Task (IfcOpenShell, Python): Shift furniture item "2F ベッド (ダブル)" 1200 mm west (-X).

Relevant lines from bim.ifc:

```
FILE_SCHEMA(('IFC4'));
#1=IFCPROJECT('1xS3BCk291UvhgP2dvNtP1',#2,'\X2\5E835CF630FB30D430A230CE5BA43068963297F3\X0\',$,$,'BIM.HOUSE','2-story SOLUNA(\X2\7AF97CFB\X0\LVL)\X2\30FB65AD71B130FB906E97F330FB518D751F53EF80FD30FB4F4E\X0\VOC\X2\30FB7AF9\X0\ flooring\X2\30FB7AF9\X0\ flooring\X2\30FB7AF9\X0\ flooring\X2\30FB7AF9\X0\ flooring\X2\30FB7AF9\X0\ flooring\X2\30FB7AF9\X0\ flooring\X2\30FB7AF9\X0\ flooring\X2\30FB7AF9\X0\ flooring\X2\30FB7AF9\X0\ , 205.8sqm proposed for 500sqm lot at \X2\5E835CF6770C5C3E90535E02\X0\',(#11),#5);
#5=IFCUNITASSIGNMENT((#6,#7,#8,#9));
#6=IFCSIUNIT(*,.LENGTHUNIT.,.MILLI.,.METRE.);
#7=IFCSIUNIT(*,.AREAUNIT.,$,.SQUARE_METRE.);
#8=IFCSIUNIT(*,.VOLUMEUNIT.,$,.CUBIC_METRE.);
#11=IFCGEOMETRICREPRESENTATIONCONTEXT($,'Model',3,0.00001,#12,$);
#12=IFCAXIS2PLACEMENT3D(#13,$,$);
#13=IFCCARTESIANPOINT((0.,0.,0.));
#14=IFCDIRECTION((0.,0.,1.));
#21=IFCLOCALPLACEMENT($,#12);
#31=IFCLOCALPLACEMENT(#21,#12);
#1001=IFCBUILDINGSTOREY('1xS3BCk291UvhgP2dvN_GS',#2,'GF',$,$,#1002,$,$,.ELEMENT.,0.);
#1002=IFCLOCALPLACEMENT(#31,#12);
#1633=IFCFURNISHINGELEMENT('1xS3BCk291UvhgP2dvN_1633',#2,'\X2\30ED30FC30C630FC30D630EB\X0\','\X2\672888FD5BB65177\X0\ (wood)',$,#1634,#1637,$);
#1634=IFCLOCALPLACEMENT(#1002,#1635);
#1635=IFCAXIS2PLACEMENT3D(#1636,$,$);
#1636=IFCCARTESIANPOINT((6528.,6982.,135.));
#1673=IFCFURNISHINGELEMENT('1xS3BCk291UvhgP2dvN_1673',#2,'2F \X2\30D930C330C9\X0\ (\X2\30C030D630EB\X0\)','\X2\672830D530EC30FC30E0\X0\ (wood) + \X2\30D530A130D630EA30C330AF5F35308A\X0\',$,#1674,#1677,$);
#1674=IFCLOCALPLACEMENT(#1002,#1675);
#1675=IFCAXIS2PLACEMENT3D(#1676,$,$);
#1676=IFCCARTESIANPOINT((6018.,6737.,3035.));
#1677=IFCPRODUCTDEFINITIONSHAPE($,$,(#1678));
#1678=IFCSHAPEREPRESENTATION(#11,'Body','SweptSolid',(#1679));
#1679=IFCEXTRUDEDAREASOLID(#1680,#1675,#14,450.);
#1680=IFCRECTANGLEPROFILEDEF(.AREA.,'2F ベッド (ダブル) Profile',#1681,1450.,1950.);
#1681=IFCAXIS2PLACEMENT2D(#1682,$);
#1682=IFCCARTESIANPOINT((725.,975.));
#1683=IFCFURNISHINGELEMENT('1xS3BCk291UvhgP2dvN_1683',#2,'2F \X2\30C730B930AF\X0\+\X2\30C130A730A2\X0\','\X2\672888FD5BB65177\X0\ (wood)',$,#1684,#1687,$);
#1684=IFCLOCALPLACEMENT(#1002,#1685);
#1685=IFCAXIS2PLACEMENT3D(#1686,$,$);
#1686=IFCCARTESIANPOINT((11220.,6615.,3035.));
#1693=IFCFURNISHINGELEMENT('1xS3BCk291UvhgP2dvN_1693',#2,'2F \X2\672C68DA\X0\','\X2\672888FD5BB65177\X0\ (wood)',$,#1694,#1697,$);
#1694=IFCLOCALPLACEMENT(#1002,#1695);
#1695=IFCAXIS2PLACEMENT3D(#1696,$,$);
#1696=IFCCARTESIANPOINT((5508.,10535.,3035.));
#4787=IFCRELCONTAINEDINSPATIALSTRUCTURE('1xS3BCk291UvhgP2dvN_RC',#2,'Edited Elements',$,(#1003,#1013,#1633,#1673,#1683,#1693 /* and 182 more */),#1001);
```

```python
import ifcopenshell
import ifcopenshell.api.geometry
import ifcopenshell.util.placement
import ifcopenshell.util.unit

model = ifcopenshell.open("bim.ifc")
unit_scale = ifcopenshell.util.unit.calculate_unit_scale(model)

item = model.by_id(1673)
matrix = ifcopenshell.util.placement.get_local_placement(item.ObjectPlacement)
matrix[0, 3] -= 1.2 / unit_scale
ifcopenshell.api.geometry.edit_object_placement(model, product=item, matrix=matrix, is_si=False)

print(ifcopenshell.util.placement.get_local_placement(item.ObjectPlacement).round(3) + 0.0)

model.write("bim_edited.ifc")
```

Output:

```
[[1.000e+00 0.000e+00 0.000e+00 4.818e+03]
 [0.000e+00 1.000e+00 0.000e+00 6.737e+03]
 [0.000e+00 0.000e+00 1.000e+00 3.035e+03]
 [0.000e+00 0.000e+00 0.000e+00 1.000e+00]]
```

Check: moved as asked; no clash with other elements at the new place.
